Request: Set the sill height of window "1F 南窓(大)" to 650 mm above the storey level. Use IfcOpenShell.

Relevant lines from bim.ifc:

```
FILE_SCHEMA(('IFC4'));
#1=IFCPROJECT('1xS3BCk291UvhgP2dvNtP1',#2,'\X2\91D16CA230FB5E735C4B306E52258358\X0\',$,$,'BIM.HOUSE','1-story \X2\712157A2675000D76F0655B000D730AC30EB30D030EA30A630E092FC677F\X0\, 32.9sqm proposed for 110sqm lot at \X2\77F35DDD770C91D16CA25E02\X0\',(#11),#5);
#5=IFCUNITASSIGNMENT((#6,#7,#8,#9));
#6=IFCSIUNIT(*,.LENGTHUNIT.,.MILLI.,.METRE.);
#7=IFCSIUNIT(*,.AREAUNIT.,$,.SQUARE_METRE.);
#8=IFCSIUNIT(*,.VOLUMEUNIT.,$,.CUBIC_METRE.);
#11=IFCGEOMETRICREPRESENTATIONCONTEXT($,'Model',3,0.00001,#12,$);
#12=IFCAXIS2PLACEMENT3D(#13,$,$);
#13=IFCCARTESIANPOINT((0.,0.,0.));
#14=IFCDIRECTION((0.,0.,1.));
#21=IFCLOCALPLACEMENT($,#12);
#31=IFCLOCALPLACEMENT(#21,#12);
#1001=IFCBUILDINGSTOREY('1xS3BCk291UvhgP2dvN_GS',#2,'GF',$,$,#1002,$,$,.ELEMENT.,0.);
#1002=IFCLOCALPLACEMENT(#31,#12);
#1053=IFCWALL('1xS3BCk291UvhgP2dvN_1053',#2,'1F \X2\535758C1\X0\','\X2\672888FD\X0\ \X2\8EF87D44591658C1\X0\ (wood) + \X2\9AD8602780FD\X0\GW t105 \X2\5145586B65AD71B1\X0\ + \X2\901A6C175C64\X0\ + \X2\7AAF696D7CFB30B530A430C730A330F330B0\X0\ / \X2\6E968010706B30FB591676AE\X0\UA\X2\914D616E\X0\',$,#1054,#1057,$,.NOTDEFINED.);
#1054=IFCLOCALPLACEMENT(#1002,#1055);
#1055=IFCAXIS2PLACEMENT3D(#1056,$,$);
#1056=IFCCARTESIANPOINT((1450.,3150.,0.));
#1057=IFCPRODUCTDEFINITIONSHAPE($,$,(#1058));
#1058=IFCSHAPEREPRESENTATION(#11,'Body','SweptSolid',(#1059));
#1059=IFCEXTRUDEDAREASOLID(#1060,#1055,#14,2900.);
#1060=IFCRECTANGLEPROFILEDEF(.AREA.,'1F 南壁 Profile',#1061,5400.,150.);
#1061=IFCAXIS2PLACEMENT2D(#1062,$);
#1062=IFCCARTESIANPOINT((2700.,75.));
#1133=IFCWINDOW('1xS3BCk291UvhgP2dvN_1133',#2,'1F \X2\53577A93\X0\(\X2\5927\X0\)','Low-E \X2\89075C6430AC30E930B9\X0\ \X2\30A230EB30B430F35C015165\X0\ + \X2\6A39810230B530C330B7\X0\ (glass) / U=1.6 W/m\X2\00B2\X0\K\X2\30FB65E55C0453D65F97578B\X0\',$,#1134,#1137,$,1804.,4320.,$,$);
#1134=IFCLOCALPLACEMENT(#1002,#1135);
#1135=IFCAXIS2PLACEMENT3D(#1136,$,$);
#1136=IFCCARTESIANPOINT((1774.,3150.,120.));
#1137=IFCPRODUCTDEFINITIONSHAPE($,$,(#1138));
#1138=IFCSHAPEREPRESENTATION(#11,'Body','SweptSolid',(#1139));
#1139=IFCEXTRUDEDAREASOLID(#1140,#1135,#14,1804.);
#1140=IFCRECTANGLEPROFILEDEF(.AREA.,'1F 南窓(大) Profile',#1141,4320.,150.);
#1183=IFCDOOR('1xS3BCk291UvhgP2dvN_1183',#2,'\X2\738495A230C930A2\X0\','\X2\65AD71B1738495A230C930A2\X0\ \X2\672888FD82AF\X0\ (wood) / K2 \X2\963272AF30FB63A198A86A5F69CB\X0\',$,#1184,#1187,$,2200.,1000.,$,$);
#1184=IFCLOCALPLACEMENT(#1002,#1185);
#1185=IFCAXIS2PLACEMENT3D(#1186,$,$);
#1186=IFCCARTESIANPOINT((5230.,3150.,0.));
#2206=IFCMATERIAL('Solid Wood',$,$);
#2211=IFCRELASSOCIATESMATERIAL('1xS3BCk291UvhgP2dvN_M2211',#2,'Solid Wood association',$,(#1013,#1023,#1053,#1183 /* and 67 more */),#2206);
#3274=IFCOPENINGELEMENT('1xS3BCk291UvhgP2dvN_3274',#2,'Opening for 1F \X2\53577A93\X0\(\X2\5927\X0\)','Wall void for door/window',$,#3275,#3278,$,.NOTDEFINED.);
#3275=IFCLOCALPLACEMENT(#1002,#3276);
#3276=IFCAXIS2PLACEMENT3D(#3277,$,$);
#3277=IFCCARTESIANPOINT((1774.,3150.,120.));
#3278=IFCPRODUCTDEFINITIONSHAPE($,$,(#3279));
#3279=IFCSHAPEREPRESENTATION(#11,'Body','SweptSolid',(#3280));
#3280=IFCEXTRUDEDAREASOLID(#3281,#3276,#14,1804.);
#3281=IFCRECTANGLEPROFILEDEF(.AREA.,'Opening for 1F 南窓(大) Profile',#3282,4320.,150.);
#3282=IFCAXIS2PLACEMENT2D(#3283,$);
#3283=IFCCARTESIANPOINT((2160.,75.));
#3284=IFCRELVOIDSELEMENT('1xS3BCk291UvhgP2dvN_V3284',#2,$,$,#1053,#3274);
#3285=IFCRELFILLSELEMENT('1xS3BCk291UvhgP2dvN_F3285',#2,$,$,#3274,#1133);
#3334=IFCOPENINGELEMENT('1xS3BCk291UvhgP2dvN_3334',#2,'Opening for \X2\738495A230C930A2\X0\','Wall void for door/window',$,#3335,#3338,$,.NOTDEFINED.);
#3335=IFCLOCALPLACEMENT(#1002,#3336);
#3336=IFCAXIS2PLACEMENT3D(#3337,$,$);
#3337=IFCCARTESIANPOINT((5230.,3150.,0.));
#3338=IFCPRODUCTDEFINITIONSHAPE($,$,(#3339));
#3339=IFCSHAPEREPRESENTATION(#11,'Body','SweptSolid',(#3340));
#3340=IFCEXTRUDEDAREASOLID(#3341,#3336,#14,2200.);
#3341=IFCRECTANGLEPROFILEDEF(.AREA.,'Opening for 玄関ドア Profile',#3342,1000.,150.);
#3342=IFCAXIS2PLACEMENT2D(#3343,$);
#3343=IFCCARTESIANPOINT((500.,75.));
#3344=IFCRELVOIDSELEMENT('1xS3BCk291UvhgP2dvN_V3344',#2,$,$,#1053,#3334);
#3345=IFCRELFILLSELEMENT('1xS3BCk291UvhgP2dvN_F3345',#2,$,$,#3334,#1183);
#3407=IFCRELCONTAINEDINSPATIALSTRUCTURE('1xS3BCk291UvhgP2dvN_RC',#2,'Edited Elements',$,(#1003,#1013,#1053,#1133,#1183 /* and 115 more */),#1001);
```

```python
import numpy as np
import ifcopenshell
import ifcopenshell.api.geometry
import ifcopenshell.geom
import ifcopenshell.util.element
import ifcopenshell.util.placement
import ifcopenshell.util.shape
import ifcopenshell.util.unit

model = ifcopenshell.open("bim.ifc")
unit_scale = ifcopenshell.util.unit.calculate_unit_scale(model)

window = model.by_guid("1xS3BCk291UvhgP2dvN_1133")
opening = window.FillsVoids[0].RelatingOpeningElement
storey = ifcopenshell.util.element.get_container(window, ifc_class="IfcBuildingStorey")
level = ifcopenshell.util.placement.get_local_placement(storey.ObjectPlacement)[2, 3]

# The opening's origin need not be at the sill, so measure its lowest point.
shape = ifcopenshell.geom.create_shape(ifcopenshell.geom.settings(), opening)
bottom = ifcopenshell.util.shape.get_shape_bottom_elevation(shape, shape.geometry) / unit_scale
dz = level + 0.65 / unit_scale - bottom

shift = np.array([0.0, 0.0, dz])
# The window is not placed relative to its opening, so move both.
for product in (opening, window):
    matrix = ifcopenshell.util.placement.get_local_placement(product.ObjectPlacement)
    matrix[:3, 3] += shift
    ifcopenshell.api.geometry.edit_object_placement(model, product=product, matrix=matrix, is_si=False)

print(f"moved by {dz * unit_scale:+.3f} m")

model.write("bim_v2.ifc")
```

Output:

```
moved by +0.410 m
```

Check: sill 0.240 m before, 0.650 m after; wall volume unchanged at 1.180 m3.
